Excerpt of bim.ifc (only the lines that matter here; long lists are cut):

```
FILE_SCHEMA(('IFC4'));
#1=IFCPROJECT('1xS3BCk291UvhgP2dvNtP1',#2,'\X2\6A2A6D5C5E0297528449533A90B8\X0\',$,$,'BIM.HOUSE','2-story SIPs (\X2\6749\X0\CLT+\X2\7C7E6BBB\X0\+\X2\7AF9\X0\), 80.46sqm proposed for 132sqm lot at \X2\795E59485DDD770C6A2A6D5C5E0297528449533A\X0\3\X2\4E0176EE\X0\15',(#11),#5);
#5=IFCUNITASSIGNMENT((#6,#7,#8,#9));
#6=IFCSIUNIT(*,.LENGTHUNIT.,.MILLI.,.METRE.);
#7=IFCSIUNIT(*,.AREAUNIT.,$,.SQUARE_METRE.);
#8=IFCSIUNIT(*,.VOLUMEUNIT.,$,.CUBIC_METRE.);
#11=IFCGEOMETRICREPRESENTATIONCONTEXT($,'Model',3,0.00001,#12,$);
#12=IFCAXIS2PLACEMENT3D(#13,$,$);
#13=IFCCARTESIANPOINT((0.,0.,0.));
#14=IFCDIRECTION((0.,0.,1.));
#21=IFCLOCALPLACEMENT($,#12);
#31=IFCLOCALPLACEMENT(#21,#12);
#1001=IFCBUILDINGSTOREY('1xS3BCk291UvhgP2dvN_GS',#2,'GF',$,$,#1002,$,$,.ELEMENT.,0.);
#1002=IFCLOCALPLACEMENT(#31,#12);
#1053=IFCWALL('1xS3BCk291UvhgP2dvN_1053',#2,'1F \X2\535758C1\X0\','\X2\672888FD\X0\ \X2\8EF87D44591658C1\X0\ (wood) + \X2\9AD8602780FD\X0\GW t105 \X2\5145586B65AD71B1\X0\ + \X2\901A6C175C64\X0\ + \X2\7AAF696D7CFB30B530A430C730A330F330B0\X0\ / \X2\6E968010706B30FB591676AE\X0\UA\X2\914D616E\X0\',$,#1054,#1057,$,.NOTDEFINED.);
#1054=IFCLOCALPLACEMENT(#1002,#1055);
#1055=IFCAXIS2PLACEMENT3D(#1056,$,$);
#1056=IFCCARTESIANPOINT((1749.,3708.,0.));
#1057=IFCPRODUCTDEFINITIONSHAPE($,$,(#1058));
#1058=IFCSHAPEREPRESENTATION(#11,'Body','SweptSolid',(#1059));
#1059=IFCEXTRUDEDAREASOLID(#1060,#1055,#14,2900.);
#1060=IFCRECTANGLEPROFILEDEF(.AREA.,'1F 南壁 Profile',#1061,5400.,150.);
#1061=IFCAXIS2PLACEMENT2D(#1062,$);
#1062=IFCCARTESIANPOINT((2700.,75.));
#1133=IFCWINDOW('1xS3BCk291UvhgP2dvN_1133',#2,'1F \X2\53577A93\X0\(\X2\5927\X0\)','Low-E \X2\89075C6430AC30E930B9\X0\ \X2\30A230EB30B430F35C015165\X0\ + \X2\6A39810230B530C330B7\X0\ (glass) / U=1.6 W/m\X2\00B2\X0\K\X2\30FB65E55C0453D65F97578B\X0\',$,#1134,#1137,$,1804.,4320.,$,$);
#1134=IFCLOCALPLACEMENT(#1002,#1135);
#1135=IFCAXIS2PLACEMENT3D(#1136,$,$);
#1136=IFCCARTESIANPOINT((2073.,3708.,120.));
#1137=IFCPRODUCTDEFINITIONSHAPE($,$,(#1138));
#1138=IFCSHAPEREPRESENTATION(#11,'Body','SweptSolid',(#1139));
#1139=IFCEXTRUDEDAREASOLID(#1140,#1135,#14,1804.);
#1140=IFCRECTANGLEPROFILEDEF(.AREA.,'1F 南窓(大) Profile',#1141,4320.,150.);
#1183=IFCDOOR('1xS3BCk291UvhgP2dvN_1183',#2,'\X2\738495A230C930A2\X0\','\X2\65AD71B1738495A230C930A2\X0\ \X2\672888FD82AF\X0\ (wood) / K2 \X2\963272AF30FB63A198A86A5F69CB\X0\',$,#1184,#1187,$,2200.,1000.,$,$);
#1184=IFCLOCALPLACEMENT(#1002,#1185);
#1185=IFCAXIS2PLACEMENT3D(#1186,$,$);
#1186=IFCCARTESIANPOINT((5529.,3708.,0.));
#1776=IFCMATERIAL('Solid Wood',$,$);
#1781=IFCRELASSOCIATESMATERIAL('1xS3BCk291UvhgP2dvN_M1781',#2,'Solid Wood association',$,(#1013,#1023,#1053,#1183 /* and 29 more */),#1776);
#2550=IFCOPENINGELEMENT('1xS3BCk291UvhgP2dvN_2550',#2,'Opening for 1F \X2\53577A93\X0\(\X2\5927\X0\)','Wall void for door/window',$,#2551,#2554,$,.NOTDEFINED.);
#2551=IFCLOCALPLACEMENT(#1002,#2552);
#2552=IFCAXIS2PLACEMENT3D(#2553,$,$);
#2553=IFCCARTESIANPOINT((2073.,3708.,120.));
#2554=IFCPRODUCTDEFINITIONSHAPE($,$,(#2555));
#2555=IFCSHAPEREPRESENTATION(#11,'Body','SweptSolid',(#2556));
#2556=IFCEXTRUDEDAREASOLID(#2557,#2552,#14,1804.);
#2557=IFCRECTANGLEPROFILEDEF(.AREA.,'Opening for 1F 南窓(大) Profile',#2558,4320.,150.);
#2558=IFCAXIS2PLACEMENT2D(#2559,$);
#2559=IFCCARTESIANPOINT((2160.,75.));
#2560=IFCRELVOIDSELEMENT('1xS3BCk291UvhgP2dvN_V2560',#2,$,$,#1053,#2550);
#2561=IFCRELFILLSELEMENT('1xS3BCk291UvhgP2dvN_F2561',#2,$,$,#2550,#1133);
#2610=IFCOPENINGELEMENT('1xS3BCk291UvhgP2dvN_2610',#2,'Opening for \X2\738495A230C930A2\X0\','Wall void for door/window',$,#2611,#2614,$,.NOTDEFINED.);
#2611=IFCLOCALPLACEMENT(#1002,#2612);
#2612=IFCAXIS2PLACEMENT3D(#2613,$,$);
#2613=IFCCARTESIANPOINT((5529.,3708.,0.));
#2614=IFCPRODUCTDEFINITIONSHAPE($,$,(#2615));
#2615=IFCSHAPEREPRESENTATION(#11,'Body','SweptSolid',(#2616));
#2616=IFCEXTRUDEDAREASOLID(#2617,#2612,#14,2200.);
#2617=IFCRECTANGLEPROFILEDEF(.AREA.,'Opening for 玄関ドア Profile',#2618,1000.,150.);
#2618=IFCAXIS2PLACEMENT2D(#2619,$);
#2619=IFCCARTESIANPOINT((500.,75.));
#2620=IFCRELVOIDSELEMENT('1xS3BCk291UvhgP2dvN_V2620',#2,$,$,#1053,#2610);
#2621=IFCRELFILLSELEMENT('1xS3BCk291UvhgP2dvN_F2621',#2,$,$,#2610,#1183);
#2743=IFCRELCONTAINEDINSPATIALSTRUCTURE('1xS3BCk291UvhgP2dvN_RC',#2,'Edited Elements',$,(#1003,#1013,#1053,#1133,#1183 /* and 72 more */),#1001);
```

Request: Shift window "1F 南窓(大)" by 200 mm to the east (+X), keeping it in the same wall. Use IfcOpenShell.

```python
import ifcopenshell
import ifcopenshell.api.geometry
import ifcopenshell.util.placement
import ifcopenshell.util.unit

model = ifcopenshell.open("bim.ifc")
unit_scale = ifcopenshell.util.unit.calculate_unit_scale(model)

window = model.by_guid("1xS3BCk291UvhgP2dvN_1133")
opening = window.FillsVoids[0].RelatingOpeningElement
wall = opening.VoidsElements[0].RelatingBuildingElement

wall_matrix = ifcopenshell.util.placement.get_local_placement(wall.ObjectPlacement)
shift = wall_matrix[:3, 0] * 0.2 / unit_scale
before = ifcopenshell.util.placement.get_local_placement(window.ObjectPlacement)[:3, 3].copy()

# The window is not placed relative to its opening, so move both.
for product in (opening, window):
    matrix = ifcopenshell.util.placement.get_local_placement(product.ObjectPlacement)
    matrix[:3, 3] += shift
    ifcopenshell.api.geometry.edit_object_placement(model, product=product, matrix=matrix, is_si=False)

after = ifcopenshell.util.placement.get_local_placement(window.ObjectPlacement)[:3, 3]
print("window moved by", (after - before).round(3) + 0.0)

model.write("bim_updated.ifc")
```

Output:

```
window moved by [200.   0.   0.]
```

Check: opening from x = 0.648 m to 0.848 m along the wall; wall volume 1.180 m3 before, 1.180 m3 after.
